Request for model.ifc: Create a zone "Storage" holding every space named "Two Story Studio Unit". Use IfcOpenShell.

First a look at what the model holds.

```python
import ifcopenshell

model = ifcopenshell.open("model.ifc")
print(model.schema)
seen = {}
for space in model.by_type("IfcSpace"):
    seen[space.LongName] = seen.get(space.LongName, 0) + 1
for name, count in sorted(seen.items(), key=str):
    print(count, "x", name)
print("zones:", [z.Name for z in model.by_type("IfcZone")][:20])
```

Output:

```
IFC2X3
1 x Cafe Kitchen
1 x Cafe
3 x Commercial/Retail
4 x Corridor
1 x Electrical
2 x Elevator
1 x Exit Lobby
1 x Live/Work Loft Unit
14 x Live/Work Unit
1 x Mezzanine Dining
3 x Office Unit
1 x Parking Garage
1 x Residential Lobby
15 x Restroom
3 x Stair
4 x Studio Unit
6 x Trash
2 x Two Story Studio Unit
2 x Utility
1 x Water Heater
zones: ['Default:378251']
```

```python
import ifcopenshell
import ifcopenshell.api.group
import ifcopenshell.api.root

model = ifcopenshell.open("model.ifc")

names = {"Two Story Studio Unit"}
spaces = [s for s in model.by_type("IfcSpace") if s.LongName in names]

zone = ifcopenshell.api.root.create_entity(model, ifc_class="IfcZone", name="Storage")
ifcopenshell.api.group.assign_group(model, products=spaces, group=zone)
print(len(spaces), "spaces in", zone.Name)

model.write("model_updated.ifc")
```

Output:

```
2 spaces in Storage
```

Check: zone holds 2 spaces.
